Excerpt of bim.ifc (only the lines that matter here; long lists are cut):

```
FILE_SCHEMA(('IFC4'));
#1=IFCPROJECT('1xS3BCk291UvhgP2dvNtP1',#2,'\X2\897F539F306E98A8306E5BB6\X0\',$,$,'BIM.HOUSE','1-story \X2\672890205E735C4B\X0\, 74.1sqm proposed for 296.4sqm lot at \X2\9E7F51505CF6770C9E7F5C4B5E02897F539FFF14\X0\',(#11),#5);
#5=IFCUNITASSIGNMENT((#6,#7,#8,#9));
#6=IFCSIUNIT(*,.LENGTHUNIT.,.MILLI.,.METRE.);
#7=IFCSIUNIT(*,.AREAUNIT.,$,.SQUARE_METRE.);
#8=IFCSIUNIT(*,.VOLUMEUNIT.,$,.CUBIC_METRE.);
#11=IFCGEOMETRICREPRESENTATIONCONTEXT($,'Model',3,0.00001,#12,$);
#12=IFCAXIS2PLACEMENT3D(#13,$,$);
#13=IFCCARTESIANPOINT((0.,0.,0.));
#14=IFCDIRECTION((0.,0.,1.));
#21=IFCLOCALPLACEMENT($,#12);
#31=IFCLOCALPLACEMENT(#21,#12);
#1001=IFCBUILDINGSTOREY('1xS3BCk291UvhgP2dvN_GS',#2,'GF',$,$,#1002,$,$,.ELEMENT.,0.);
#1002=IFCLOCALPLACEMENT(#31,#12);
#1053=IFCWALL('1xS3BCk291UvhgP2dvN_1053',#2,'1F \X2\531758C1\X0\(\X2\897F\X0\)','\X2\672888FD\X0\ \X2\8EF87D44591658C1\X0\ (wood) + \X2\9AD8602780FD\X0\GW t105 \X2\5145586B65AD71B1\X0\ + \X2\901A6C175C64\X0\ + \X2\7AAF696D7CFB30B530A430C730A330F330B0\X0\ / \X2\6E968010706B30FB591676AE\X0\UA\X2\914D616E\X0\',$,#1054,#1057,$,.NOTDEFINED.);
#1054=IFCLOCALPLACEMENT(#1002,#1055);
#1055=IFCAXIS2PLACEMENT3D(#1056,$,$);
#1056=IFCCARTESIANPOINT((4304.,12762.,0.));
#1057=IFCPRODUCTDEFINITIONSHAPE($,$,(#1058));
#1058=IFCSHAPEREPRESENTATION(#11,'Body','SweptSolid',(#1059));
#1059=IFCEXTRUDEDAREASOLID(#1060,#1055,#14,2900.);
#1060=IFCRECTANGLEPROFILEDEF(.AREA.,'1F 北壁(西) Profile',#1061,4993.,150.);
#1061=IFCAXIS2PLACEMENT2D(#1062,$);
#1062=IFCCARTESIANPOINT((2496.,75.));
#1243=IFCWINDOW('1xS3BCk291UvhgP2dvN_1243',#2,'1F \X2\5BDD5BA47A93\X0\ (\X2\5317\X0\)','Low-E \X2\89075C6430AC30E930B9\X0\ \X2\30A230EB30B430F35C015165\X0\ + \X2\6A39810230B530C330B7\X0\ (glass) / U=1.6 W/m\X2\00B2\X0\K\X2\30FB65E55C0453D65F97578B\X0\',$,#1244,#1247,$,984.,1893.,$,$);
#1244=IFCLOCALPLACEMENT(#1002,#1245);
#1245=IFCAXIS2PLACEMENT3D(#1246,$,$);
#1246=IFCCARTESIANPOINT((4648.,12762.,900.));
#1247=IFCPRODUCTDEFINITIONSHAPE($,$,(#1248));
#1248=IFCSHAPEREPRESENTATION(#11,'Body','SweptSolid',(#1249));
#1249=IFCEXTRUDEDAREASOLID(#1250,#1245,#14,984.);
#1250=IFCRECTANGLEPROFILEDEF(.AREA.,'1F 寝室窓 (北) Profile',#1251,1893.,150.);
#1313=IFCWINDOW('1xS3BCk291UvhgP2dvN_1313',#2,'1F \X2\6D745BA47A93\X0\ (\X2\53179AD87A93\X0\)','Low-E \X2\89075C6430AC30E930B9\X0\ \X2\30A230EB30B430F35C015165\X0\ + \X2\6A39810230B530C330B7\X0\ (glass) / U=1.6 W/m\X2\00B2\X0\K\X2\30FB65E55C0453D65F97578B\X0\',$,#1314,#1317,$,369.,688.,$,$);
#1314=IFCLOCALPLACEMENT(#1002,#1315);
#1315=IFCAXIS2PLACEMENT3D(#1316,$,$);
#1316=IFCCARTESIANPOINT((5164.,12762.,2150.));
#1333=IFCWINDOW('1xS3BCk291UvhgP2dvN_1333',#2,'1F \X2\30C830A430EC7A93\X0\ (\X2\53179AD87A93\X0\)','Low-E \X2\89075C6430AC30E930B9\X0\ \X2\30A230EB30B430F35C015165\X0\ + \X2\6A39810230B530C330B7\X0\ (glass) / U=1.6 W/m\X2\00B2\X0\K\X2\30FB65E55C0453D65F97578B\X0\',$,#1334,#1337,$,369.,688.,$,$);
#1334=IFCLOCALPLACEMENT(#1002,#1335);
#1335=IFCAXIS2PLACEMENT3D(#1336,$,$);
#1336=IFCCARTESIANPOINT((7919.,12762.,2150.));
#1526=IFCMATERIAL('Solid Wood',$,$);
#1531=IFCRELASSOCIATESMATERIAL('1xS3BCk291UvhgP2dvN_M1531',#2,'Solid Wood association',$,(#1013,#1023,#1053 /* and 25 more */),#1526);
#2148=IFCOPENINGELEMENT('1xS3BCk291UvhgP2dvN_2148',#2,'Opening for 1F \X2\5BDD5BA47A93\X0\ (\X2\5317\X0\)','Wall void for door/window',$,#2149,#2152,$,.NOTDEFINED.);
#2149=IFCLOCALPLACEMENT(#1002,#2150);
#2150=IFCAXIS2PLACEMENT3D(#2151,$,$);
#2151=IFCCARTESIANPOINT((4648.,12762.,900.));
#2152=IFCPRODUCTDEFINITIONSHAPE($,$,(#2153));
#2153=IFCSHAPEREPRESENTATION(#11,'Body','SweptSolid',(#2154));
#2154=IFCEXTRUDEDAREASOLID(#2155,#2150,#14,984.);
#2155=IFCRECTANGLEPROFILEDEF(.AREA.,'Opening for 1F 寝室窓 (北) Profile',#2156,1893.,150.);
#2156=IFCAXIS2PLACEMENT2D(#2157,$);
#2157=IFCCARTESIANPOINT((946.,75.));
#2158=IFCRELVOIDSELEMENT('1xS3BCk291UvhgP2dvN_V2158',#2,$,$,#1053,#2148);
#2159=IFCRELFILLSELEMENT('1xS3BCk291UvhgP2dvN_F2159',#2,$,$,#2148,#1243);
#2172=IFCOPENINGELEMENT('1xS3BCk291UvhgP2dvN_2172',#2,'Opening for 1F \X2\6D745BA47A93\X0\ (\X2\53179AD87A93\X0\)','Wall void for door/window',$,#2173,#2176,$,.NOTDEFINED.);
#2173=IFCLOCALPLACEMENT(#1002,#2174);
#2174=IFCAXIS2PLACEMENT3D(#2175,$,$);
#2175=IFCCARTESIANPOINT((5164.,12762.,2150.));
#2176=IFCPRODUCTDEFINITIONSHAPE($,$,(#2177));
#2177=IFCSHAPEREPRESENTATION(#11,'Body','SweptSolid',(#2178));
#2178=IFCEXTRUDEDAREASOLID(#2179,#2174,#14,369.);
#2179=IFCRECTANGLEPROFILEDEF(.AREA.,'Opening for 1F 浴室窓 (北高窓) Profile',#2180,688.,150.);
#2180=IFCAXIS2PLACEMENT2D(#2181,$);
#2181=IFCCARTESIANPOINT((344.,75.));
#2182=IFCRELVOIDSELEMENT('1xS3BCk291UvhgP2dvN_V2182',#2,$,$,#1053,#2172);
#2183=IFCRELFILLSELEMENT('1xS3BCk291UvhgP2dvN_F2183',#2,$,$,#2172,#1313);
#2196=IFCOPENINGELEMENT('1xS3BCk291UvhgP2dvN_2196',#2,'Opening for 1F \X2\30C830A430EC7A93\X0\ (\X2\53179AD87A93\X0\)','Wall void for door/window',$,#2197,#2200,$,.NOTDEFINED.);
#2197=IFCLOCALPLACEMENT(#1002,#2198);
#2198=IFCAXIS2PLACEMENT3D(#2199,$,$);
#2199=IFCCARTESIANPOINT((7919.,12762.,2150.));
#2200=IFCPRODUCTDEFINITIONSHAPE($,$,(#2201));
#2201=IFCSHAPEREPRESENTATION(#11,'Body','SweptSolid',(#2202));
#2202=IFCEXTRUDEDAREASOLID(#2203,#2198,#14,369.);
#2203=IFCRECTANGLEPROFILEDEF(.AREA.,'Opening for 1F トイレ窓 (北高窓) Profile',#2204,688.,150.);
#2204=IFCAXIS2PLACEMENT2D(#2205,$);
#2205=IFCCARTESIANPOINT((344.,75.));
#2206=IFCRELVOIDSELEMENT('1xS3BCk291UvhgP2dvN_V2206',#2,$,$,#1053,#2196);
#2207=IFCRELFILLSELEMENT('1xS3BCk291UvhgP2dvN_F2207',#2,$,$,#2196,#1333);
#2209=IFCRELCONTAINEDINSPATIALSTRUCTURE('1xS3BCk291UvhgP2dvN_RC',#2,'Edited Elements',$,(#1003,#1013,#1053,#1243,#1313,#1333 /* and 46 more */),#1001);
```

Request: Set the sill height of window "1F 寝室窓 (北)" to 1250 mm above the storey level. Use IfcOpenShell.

```python
import numpy as np
import ifcopenshell
import ifcopenshell.api.geometry
import ifcopenshell.geom
import ifcopenshell.util.element
import ifcopenshell.util.placement
import ifcopenshell.util.shape
import ifcopenshell.util.unit

model = ifcopenshell.open("bim.ifc")
unit_scale = ifcopenshell.util.unit.calculate_unit_scale(model)

window = model.by_id(1243)
opening = window.FillsVoids[0].RelatingOpeningElement
storey = ifcopenshell.util.element.get_container(window, ifc_class="IfcBuildingStorey")
level = ifcopenshell.util.placement.get_local_placement(storey.ObjectPlacement)[2, 3]

# The opening's origin need not be at the sill, so measure its lowest point.
shape = ifcopenshell.geom.create_shape(ifcopenshell.geom.settings(), opening)
bottom = ifcopenshell.util.shape.get_shape_bottom_elevation(shape, shape.geometry) / unit_scale
dz = level + 1250.0 - bottom

shift = np.array([0.0, 0.0, dz])
# The window is not placed relative to its opening, so move both.
for product in (opening, window):
    matrix = ifcopenshell.util.placement.get_local_placement(product.ObjectPlacement)
    matrix[:3, 3] += shift
    ifcopenshell.api.geometry.edit_object_placement(model, product=product, matrix=matrix, is_si=False)

print(f"moved by {dz * unit_scale:+.3f} m")

model.write("bim-out.ifc")
```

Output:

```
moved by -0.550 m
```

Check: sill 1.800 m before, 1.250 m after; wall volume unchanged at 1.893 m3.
